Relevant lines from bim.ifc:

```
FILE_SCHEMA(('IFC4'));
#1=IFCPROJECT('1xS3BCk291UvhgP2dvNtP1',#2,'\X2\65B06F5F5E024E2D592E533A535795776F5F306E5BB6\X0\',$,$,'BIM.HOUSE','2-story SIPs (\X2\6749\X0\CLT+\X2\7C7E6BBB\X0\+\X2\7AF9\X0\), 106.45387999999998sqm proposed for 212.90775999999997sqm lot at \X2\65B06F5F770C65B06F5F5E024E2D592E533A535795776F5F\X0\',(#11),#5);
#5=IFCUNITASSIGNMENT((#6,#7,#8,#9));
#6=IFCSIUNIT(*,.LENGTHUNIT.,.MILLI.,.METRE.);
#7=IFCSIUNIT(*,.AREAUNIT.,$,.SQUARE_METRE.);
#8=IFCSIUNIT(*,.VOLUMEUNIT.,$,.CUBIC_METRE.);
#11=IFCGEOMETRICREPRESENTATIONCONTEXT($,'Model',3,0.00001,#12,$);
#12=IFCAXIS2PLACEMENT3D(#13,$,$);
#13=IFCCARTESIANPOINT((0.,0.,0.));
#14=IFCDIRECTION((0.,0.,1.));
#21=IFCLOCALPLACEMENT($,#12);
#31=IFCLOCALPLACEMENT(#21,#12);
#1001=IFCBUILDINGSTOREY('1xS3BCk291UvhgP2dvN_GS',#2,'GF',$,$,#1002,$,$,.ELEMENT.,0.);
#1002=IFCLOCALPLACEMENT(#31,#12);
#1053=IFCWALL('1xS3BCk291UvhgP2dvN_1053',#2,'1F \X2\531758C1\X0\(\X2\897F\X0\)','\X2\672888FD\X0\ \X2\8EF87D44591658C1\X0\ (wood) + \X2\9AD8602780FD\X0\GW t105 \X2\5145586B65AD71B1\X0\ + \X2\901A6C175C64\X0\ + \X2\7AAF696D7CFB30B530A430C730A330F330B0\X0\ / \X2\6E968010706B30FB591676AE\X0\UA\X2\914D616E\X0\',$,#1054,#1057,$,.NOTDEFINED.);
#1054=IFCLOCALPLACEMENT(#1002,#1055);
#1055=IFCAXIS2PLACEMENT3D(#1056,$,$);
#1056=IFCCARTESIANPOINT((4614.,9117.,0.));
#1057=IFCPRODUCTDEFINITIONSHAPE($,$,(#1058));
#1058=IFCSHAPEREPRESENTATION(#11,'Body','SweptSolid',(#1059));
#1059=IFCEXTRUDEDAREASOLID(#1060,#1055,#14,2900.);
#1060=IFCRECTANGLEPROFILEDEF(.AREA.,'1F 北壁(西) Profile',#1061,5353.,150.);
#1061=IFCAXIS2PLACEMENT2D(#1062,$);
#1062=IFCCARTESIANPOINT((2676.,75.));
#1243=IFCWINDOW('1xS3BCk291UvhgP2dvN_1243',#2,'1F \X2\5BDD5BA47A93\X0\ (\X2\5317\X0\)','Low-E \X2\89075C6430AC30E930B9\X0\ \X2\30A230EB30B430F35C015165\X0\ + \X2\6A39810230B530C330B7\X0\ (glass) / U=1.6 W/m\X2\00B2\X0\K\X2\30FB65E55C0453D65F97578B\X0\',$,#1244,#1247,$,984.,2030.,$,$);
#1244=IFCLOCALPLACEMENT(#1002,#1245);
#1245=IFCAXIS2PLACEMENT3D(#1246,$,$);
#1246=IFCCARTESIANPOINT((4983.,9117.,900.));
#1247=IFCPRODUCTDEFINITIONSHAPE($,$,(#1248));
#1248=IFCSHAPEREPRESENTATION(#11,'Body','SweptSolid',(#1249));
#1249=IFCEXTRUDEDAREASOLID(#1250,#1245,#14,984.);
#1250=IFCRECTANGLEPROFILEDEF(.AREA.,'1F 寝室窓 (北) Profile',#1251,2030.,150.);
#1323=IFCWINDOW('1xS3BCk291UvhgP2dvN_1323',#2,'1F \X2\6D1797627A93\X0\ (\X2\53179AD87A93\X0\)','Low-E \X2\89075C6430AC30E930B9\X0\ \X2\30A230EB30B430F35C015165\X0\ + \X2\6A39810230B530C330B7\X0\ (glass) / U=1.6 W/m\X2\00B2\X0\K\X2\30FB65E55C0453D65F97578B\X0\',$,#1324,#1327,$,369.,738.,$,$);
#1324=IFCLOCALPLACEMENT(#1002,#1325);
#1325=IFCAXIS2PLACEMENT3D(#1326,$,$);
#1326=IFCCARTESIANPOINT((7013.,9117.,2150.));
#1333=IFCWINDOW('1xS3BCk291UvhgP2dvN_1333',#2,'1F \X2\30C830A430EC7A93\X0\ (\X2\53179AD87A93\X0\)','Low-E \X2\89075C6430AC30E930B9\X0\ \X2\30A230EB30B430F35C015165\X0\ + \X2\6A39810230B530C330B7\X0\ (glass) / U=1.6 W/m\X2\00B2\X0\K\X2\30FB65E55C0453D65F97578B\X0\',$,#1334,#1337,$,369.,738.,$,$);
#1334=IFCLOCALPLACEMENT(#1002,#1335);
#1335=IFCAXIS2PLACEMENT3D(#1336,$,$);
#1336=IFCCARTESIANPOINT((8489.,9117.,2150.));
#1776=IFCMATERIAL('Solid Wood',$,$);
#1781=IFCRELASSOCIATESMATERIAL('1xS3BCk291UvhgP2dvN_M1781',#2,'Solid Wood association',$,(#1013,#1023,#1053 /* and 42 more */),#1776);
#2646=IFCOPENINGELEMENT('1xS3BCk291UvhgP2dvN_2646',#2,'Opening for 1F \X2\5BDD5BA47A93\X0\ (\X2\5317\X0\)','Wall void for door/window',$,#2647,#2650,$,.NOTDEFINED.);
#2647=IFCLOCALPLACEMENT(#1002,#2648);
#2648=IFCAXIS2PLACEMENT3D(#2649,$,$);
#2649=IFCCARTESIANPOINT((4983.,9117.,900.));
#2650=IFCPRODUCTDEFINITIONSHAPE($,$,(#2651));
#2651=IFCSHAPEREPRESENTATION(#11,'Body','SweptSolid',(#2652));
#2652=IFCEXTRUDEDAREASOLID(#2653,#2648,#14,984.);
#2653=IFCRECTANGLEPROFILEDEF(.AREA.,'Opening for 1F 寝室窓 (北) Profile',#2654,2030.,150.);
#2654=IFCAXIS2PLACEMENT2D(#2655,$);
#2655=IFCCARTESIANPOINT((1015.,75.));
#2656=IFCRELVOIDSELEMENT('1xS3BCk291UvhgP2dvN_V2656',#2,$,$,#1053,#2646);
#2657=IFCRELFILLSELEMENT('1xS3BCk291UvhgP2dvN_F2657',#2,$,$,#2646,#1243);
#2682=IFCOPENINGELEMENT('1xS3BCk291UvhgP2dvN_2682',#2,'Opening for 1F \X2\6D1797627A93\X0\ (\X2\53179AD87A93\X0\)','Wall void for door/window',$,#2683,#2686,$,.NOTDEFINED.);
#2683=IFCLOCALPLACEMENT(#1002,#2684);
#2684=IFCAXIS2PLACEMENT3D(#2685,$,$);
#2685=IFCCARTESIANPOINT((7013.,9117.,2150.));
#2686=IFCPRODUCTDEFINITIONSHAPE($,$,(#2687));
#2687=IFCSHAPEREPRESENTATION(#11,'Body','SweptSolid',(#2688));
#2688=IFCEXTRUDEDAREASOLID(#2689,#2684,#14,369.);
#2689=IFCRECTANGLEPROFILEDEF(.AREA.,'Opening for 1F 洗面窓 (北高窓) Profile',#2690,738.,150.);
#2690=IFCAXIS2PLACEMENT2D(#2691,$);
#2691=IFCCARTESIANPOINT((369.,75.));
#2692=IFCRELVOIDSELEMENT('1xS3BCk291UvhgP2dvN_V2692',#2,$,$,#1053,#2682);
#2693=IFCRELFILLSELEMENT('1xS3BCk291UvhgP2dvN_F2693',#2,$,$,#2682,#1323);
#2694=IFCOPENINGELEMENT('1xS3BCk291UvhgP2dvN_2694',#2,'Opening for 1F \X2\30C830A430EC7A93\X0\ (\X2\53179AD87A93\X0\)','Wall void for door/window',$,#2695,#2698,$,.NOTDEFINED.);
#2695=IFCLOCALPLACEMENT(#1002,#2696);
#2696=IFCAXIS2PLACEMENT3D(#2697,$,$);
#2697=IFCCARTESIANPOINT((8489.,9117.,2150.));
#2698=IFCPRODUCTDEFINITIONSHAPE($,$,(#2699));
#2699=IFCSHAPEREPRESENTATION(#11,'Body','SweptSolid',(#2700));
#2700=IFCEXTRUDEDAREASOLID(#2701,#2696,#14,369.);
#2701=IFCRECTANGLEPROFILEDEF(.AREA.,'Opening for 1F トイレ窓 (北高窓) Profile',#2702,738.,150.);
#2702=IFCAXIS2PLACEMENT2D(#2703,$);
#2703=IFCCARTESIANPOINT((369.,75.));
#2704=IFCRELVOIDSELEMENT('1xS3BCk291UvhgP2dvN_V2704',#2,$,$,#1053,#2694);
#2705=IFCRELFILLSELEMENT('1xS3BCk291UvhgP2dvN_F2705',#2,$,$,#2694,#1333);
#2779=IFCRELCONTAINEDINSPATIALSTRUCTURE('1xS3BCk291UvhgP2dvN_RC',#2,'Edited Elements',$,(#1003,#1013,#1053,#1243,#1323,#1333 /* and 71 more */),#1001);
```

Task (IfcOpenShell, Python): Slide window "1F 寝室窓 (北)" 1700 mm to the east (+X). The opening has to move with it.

```python
import ifcopenshell
import ifcopenshell.api.geometry
import ifcopenshell.util.placement
import ifcopenshell.util.unit

model = ifcopenshell.open("bim.ifc")
unit_scale = ifcopenshell.util.unit.calculate_unit_scale(model)

window = model.by_guid("1xS3BCk291UvhgP2dvN_1243")
opening = window.FillsVoids[0].RelatingOpeningElement
wall = opening.VoidsElements[0].RelatingBuildingElement

wall_matrix = ifcopenshell.util.placement.get_local_placement(wall.ObjectPlacement)
shift = wall_matrix[:3, 0] * 1.7 / unit_scale
before = ifcopenshell.util.placement.get_local_placement(window.ObjectPlacement)[:3, 3].copy()

# The window is not placed relative to its opening, so move both.
for product in (opening, window):
    matrix = ifcopenshell.util.placement.get_local_placement(product.ObjectPlacement)
    matrix[:3, 3] += shift
    ifcopenshell.api.geometry.edit_object_placement(model, product=product, matrix=matrix, is_si=False)

after = ifcopenshell.util.placement.get_local_placement(window.ObjectPlacement)[:3, 3]
print("window moved by", (after - before).round(3) + 0.0)

model.write("bim_updated.ifc")
```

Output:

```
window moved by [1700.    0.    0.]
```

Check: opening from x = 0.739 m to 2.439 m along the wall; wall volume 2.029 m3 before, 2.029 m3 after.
